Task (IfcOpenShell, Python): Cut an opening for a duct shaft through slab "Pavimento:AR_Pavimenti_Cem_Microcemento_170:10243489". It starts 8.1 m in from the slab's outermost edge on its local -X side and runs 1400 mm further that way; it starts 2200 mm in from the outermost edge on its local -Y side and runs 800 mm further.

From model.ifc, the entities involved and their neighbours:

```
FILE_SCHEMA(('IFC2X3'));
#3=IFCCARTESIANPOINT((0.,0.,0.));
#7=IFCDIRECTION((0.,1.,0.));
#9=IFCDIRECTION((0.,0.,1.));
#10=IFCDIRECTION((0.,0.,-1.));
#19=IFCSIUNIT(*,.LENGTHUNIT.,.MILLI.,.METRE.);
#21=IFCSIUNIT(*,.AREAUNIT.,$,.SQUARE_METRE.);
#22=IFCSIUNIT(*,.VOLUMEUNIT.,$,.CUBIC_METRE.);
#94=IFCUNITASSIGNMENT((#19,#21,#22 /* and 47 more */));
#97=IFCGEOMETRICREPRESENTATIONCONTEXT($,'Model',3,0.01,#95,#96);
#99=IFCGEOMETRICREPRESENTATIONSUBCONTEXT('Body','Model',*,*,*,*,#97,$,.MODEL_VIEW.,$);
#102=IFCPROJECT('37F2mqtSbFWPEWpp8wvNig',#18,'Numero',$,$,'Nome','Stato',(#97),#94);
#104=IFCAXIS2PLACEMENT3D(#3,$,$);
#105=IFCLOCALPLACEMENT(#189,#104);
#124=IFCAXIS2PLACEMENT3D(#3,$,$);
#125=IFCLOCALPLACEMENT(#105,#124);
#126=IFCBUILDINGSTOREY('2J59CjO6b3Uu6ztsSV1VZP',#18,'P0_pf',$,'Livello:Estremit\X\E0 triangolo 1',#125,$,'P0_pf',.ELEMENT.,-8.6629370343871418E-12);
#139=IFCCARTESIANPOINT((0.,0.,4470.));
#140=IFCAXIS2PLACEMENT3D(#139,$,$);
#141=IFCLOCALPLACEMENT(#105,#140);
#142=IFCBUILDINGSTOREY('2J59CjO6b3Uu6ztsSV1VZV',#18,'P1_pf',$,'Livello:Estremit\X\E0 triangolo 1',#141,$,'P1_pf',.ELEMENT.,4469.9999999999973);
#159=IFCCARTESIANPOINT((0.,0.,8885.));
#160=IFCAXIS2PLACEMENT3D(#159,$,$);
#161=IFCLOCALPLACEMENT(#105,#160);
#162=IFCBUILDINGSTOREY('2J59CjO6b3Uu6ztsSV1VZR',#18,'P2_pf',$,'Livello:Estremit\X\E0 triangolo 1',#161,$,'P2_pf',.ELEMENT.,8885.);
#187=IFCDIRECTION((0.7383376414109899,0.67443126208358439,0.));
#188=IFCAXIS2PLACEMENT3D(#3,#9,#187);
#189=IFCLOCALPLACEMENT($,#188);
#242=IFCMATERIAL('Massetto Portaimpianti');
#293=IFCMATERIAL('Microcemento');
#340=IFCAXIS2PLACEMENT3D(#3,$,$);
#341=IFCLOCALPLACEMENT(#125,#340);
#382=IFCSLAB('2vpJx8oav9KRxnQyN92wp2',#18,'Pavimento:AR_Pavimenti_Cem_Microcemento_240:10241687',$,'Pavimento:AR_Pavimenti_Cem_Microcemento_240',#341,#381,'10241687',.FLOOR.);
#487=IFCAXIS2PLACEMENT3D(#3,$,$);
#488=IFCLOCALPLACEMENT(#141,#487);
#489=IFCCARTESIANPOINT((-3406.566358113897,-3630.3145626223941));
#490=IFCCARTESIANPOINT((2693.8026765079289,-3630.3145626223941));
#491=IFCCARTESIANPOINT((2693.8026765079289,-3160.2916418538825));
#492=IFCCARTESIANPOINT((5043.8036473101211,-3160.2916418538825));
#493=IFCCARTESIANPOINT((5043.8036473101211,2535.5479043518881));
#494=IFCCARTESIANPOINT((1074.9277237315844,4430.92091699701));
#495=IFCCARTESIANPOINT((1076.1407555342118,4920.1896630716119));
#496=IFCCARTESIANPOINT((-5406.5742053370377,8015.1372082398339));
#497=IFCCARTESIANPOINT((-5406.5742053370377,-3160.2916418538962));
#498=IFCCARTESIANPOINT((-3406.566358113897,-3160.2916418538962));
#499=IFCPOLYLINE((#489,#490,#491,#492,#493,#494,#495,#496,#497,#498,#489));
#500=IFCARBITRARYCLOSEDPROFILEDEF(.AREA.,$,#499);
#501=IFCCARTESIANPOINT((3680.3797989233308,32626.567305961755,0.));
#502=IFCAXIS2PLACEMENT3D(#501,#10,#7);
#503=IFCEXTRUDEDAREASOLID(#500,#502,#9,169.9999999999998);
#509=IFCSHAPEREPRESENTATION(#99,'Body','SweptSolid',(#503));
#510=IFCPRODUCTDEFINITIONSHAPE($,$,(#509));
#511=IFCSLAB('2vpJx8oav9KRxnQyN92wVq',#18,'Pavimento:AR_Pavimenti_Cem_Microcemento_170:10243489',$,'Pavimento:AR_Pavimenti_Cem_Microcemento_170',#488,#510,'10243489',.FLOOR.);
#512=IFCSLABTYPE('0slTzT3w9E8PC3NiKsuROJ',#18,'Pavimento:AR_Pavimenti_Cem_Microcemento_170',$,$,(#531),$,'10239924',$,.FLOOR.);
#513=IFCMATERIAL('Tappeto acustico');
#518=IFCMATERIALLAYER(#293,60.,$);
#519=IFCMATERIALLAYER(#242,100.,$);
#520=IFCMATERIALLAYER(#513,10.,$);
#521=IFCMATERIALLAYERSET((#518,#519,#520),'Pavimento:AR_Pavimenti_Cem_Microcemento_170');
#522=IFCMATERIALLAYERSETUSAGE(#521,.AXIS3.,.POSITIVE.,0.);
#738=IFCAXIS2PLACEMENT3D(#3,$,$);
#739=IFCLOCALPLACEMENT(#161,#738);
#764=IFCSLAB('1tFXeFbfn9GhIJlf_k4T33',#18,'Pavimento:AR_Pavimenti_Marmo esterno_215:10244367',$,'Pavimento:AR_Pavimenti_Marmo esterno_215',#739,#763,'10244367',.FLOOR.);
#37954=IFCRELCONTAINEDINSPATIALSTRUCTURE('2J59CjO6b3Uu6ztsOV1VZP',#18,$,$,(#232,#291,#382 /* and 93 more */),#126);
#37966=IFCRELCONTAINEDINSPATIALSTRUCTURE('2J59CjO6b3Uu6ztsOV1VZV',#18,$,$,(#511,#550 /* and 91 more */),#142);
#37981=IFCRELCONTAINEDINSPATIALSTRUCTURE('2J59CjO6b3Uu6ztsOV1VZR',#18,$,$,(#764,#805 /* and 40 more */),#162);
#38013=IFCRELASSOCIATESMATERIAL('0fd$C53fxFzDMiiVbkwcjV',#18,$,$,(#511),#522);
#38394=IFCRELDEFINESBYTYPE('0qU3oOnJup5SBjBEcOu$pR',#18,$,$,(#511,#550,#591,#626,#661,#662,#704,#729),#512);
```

```python
import numpy as np
import ifcopenshell
import ifcopenshell.api.feature
import ifcopenshell.api.geometry
import ifcopenshell.api.root
import ifcopenshell.geom
import ifcopenshell.util.placement
import ifcopenshell.util.representation
import ifcopenshell.util.shape
import ifcopenshell.util.unit

model = ifcopenshell.open("model.ifc")
unit_scale = ifcopenshell.util.unit.calculate_unit_scale(model)
settings = ifcopenshell.geom.settings()


def volume(element):
    """Net volume in cubic metres, openings subtracted."""
    shape = ifcopenshell.geom.create_shape(settings, element)
    return ifcopenshell.util.shape.get_volume(shape.geometry)


slab = model.by_guid("2vpJx8oav9KRxnQyN92wVq")
before = volume(slab)

# Extent in the slab's own axes, in metres. The edges named are its -X and -Y sides.
slab_shape = ifcopenshell.geom.create_shape(settings, slab)
vertices = ifcopenshell.util.shape.get_vertices(slab_shape.geometry)
x_min, y_min, bottom = vertices.min(axis=0)
top = vertices[:, 2].max()

opening = ifcopenshell.api.root.create_entity(model, ifc_class="IfcOpeningElement", name="Duct shaft opening")
context = ifcopenshell.util.representation.get_context(model, "Model", "Body", "MODEL_VIEW")
width, depth = 1.4, 0.8
outline = [(0.0, 0.0), (width, 0.0), (width, depth), (0.0, depth), (0.0, 0.0)]
# Overshoot both faces by 50 mm so the cut is clean.
shape = ifcopenshell.api.geometry.add_slab_representation(
    model, context=context, depth=top - bottom + 0.1, polyline=outline
)
ifcopenshell.api.geometry.assign_representation(model, product=opening, representation=shape)

matrix = ifcopenshell.util.placement.get_local_placement(slab.ObjectPlacement)
matrix[:, 3] = matrix @ np.append(np.array([x_min + 8.1, y_min + 2.2, bottom - 0.05]) / unit_scale, 1.0)
ifcopenshell.api.geometry.edit_object_placement(model, product=opening, matrix=matrix, is_si=False)
ifcopenshell.api.feature.add_feature(model, feature=opening, element=slab)

after = volume(slab)

print(f"slab volume {before:.3f} -> {after:.3f} m3")

model.write("model_edited.ifc")
```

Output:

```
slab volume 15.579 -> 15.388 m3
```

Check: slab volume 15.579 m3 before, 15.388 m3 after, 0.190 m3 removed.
